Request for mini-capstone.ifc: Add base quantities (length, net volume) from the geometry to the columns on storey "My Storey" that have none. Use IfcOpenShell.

First a look at what the model holds.

```python
import ifcopenshell
import ifcopenshell.util.element
import ifcopenshell.util.unit

model = ifcopenshell.open("mini-capstone.ifc")
print(model.schema)
for unit_type in ("LENGTHUNIT", "AREAUNIT", "VOLUMEUNIT"):
    print(unit_type, ifcopenshell.util.unit.calculate_unit_scale(model, unit_type))
storey = next(s for s in model.by_type("IfcBuildingStorey") if s.Name == "My Storey")
columns = [e for e in ifcopenshell.util.element.get_decomposition(storey) if e.is_a("IfcColumn")]
for e in sorted(columns, key=lambda e: e.id()):
    print(e.id(), e.is_a(), e.Name, list(ifcopenshell.util.element.get_psets(e, qtos_only=True)), sep=" | ")
```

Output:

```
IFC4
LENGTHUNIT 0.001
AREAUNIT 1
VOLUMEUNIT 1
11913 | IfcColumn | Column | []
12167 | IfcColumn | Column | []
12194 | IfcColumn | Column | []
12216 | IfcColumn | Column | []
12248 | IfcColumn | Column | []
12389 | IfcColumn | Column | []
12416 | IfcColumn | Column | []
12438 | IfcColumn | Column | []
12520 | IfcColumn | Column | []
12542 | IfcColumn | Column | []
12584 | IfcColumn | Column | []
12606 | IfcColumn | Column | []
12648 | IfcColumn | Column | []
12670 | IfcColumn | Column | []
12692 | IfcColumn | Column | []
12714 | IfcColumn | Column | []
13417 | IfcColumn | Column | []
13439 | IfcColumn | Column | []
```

```python
import ifcopenshell
import ifcopenshell.api.pset
import ifcopenshell.geom
import ifcopenshell.util.element
import ifcopenshell.util.shape
import ifcopenshell.util.unit

model = ifcopenshell.open("mini-capstone.ifc")
unit_scale = ifcopenshell.util.unit.calculate_unit_scale(model)
volume_scale = ifcopenshell.util.unit.calculate_unit_scale(model, "VOLUMEUNIT")
settings = ifcopenshell.geom.settings()

storey = next(s for s in model.by_type("IfcBuildingStorey") if s.Name == "My Storey")
columns = [e for e in ifcopenshell.util.element.get_decomposition(storey) if e.is_a("IfcColumn")]

for e in sorted(columns, key=lambda e: e.id()):
    if ifcopenshell.util.element.get_psets(e, qtos_only=True, should_inherit=False):
        continue
    # Geometry comes back in metres, in the element's own axes.
    shape = ifcopenshell.geom.create_shape(settings, e)
    values = {
        "Length": ifcopenshell.util.shape.get_z(shape.geometry) / unit_scale,
        "NetVolume": ifcopenshell.util.shape.get_volume(shape.geometry) / volume_scale,
    }
    qto = ifcopenshell.api.pset.add_qto(model, product=e, name="Qto_ColumnBaseQuantities")
    ifcopenshell.api.pset.edit_qto(model, qto=qto, properties=values)
    print(e.id(), {k: round(v, 3) for k, v in values.items()})

model.write("mini-capstone_rev.ifc")
```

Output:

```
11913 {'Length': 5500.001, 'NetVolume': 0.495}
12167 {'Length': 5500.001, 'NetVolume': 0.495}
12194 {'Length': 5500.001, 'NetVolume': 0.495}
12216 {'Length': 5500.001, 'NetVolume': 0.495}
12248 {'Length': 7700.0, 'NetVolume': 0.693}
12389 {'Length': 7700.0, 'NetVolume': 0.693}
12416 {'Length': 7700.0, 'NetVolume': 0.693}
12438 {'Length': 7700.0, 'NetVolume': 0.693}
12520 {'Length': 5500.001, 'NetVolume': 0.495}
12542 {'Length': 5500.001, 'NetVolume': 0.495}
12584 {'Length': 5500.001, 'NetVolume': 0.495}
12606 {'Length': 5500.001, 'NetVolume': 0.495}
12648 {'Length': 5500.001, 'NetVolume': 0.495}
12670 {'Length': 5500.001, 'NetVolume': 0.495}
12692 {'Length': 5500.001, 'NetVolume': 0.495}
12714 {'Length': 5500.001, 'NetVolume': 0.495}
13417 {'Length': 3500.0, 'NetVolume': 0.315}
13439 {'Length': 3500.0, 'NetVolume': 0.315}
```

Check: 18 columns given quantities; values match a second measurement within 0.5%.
